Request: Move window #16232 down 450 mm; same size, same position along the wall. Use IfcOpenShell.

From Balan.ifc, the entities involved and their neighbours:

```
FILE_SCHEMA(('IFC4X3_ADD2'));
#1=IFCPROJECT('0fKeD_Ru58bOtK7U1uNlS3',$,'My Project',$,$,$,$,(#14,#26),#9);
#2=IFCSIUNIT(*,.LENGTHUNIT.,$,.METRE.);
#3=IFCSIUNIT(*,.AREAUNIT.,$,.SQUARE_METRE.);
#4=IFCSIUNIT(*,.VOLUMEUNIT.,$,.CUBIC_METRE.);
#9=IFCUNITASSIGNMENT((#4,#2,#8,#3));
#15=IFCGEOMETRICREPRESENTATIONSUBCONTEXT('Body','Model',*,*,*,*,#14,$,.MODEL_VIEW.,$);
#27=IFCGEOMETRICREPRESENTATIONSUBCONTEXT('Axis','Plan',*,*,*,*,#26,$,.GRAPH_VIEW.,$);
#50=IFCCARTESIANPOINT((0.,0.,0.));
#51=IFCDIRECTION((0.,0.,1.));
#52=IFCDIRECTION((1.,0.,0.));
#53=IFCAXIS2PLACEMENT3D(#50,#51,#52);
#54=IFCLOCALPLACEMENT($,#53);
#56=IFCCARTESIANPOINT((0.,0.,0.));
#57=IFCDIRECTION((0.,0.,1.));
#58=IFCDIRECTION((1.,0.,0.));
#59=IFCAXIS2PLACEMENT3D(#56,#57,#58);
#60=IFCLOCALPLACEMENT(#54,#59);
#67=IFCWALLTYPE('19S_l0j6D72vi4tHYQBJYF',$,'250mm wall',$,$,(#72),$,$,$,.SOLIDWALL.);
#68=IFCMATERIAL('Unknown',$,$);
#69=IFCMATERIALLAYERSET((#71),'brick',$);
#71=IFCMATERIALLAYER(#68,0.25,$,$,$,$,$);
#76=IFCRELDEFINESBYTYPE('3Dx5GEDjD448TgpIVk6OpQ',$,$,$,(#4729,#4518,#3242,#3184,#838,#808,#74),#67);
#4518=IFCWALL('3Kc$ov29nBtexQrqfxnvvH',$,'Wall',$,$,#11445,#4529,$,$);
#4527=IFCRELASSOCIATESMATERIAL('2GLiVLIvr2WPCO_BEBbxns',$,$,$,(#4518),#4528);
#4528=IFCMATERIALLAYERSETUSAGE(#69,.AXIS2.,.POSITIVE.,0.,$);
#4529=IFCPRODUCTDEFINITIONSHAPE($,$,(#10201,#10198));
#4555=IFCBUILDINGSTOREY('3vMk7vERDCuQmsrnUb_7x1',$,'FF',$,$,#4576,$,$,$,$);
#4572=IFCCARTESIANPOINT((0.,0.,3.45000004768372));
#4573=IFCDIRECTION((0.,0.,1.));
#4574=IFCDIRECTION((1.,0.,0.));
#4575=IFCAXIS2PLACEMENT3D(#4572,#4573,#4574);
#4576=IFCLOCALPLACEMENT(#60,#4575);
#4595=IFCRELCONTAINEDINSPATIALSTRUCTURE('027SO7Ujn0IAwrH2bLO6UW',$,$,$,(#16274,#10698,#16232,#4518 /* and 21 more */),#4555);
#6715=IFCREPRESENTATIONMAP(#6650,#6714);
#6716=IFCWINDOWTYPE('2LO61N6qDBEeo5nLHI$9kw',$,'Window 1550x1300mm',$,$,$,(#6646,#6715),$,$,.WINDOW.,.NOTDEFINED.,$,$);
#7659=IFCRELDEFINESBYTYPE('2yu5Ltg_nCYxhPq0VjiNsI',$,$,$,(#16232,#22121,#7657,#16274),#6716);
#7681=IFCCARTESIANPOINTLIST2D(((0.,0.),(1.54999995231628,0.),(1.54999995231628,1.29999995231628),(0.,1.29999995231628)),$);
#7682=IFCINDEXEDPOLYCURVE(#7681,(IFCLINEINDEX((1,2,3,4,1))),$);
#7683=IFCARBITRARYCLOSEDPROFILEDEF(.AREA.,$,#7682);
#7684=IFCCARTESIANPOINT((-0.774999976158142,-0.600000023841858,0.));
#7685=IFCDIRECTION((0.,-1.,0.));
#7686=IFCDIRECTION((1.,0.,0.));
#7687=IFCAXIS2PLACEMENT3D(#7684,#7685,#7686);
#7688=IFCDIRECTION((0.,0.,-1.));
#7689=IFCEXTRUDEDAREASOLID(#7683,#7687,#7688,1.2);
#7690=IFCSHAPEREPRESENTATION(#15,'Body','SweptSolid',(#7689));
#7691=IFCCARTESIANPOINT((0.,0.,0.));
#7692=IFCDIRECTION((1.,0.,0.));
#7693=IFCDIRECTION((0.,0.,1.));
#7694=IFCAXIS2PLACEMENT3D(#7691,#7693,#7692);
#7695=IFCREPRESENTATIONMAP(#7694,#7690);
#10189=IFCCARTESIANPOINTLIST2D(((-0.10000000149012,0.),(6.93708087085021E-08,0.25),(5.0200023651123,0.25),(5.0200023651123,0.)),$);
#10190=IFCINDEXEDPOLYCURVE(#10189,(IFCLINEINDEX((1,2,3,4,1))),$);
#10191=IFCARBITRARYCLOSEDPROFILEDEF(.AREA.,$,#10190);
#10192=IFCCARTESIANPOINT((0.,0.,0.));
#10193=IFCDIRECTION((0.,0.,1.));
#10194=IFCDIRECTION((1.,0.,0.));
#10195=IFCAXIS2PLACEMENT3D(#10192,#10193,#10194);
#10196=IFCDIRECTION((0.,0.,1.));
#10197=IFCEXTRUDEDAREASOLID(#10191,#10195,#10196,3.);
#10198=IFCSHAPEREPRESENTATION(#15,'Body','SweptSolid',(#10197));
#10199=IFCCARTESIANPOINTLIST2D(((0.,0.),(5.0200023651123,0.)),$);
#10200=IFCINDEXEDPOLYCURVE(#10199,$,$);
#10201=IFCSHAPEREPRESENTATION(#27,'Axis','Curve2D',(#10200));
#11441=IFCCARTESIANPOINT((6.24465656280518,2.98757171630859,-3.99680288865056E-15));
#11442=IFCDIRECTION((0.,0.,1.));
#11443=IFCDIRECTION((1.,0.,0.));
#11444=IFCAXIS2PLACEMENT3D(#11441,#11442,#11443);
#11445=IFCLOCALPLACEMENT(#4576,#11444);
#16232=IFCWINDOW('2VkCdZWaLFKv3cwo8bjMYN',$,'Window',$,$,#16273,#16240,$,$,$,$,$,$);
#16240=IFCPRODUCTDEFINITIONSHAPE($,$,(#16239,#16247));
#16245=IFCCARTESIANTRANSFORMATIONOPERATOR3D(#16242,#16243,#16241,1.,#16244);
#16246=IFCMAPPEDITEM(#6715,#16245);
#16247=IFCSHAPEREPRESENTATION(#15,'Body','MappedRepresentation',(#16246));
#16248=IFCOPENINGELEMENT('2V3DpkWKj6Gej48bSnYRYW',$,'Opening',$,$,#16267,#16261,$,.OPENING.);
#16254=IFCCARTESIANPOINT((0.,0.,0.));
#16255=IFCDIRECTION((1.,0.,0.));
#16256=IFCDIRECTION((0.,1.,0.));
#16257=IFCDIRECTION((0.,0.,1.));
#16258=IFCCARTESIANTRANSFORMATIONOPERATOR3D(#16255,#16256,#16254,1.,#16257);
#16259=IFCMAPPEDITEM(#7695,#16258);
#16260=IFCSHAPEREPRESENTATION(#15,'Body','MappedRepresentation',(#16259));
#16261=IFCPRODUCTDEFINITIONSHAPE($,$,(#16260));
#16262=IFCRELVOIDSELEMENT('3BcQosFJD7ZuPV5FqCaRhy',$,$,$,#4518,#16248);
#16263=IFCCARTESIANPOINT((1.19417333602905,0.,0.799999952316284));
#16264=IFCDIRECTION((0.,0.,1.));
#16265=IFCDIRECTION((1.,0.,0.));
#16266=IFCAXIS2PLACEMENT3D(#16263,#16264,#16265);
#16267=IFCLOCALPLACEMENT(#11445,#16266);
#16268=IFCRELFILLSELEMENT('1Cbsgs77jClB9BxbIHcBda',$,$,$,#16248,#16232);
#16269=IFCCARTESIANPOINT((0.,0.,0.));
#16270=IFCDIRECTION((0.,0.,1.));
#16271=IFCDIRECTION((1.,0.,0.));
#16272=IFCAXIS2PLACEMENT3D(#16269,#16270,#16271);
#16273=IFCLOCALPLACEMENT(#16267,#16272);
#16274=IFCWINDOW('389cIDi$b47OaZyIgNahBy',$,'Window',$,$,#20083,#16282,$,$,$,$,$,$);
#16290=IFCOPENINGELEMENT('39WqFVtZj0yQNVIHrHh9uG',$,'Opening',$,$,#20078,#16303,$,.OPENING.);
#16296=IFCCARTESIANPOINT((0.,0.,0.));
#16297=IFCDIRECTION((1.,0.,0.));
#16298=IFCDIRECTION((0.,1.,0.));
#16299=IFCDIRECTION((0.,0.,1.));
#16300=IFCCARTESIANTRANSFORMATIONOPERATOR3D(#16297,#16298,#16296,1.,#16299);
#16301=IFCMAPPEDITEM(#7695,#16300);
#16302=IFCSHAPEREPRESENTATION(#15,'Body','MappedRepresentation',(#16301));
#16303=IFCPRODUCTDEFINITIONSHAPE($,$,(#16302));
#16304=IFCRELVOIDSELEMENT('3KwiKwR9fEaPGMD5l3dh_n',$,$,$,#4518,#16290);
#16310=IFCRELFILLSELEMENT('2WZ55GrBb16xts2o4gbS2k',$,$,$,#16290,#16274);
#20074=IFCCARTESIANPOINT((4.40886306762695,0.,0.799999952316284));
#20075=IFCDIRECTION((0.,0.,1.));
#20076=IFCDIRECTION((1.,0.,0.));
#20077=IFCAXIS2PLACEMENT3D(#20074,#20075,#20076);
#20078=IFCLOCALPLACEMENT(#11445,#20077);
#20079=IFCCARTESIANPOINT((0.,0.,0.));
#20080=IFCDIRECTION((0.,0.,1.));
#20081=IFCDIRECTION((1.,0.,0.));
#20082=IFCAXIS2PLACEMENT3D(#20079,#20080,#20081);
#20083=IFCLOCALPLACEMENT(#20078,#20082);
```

```python
import numpy as np
import ifcopenshell
import ifcopenshell.api.geometry
import ifcopenshell.util.placement
import ifcopenshell.util.unit

model = ifcopenshell.open("Balan.ifc")
unit_scale = ifcopenshell.util.unit.calculate_unit_scale(model)

window = model.by_id(16232)
opening = window.FillsVoids[0].RelatingOpeningElement
dz = -0.45

shift = np.array([0.0, 0.0, dz])
# The window is placed relative to its opening, so it follows when the opening moves.
matrix = ifcopenshell.util.placement.get_local_placement(opening.ObjectPlacement)
matrix[:3, 3] += shift
ifcopenshell.api.geometry.edit_object_placement(
    model, product=opening, matrix=matrix, is_si=False, should_transform_children=True
)

print(f"moved by {dz * unit_scale:+.3f} m")

model.write("Balan-out.ifc")
```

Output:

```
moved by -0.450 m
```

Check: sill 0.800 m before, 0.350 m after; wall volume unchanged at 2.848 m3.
